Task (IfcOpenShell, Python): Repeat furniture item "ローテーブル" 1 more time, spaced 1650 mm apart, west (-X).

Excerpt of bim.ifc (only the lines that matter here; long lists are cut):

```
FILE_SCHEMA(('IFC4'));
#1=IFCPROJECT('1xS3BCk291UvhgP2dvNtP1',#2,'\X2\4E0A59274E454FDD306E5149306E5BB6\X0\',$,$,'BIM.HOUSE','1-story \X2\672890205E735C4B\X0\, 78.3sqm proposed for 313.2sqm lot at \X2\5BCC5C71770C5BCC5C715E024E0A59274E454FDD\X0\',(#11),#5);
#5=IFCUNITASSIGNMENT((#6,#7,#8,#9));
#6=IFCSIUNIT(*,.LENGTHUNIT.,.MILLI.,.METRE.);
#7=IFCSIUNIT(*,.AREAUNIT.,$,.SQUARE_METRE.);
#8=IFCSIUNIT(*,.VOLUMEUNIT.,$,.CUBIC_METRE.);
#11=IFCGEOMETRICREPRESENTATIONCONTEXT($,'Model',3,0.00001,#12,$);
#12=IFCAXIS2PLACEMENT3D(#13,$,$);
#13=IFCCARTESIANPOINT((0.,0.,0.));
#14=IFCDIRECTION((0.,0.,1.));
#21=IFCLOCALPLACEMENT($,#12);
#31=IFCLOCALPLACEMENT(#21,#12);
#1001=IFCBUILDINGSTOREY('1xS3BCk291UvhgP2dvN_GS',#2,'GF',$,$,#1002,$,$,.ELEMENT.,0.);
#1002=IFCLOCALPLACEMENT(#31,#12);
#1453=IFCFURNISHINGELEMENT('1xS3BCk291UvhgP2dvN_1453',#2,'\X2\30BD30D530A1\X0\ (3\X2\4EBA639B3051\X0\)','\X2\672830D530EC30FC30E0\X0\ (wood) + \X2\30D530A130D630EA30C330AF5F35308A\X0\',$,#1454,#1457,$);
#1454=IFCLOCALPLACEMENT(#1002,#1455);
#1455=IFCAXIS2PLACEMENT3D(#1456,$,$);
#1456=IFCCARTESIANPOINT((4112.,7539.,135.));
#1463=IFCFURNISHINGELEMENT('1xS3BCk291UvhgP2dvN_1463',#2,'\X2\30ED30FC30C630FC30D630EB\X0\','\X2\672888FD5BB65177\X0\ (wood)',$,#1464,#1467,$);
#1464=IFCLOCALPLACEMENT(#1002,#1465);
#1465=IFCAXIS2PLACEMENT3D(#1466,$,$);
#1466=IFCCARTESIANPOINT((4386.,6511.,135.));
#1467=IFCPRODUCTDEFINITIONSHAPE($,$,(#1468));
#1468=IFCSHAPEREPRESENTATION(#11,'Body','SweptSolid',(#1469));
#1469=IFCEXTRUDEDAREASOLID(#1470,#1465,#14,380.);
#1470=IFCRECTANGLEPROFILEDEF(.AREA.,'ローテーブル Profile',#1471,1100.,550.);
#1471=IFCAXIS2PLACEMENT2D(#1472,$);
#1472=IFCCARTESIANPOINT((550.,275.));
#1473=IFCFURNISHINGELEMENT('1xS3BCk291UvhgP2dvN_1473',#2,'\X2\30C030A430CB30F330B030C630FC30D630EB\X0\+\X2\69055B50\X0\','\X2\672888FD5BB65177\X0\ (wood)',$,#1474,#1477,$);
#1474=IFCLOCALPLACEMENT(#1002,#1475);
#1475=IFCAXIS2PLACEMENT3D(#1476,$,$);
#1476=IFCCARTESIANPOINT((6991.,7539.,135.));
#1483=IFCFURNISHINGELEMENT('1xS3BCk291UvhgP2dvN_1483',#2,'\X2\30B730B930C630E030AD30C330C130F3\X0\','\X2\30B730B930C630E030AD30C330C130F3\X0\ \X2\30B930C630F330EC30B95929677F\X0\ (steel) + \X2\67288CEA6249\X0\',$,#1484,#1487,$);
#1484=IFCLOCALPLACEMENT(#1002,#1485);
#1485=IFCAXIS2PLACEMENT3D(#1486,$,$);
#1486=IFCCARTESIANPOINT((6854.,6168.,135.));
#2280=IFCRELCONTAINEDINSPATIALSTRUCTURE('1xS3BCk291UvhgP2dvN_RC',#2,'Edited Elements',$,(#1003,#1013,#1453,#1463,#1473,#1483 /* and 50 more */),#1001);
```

```python
import numpy as np
import ifcopenshell
import ifcopenshell.api.geometry
import ifcopenshell.api.root
import ifcopenshell.util.element
import ifcopenshell.util.placement

model = ifcopenshell.open("bim.ifc")


def reuse_history(source, copy):
    """copy_class also copies each property set's owner history, people and application; keep the originals."""
    for rel in copy.IsDefinedBy:
        if rel.is_a("IfcRelDefinesByProperties") and (history := rel.RelatingPropertyDefinition.OwnerHistory):
            rel.RelatingPropertyDefinition.OwnerHistory = source.OwnerHistory
            ifcopenshell.util.element.remove_deep2(model, history)


source = model.by_guid("1xS3BCk291UvhgP2dvN_1463")
base = ifcopenshell.util.placement.get_local_placement(source.ObjectPlacement)
step = np.array([-1.0, 0.0, 0.0]) * 1650.0

for i in range(1, 2):
    copy = ifcopenshell.api.root.copy_class(model, product=source)
    copy.Representation = ifcopenshell.util.element.copy_deep(
        model, source.Representation, exclude=["IfcGeometricRepresentationContext", "IfcRepresentationMap"]
    )
    reuse_history(source, copy)
    matrix = base.copy()
    matrix[:3, 3] += i * step
    print("added at", matrix[:3, 3].round(3) + 0.0)
    ifcopenshell.api.geometry.edit_object_placement(model, product=copy, matrix=matrix, is_si=False)

model.write("bim-out.ifc")
```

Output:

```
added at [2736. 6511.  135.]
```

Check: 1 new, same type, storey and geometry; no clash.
